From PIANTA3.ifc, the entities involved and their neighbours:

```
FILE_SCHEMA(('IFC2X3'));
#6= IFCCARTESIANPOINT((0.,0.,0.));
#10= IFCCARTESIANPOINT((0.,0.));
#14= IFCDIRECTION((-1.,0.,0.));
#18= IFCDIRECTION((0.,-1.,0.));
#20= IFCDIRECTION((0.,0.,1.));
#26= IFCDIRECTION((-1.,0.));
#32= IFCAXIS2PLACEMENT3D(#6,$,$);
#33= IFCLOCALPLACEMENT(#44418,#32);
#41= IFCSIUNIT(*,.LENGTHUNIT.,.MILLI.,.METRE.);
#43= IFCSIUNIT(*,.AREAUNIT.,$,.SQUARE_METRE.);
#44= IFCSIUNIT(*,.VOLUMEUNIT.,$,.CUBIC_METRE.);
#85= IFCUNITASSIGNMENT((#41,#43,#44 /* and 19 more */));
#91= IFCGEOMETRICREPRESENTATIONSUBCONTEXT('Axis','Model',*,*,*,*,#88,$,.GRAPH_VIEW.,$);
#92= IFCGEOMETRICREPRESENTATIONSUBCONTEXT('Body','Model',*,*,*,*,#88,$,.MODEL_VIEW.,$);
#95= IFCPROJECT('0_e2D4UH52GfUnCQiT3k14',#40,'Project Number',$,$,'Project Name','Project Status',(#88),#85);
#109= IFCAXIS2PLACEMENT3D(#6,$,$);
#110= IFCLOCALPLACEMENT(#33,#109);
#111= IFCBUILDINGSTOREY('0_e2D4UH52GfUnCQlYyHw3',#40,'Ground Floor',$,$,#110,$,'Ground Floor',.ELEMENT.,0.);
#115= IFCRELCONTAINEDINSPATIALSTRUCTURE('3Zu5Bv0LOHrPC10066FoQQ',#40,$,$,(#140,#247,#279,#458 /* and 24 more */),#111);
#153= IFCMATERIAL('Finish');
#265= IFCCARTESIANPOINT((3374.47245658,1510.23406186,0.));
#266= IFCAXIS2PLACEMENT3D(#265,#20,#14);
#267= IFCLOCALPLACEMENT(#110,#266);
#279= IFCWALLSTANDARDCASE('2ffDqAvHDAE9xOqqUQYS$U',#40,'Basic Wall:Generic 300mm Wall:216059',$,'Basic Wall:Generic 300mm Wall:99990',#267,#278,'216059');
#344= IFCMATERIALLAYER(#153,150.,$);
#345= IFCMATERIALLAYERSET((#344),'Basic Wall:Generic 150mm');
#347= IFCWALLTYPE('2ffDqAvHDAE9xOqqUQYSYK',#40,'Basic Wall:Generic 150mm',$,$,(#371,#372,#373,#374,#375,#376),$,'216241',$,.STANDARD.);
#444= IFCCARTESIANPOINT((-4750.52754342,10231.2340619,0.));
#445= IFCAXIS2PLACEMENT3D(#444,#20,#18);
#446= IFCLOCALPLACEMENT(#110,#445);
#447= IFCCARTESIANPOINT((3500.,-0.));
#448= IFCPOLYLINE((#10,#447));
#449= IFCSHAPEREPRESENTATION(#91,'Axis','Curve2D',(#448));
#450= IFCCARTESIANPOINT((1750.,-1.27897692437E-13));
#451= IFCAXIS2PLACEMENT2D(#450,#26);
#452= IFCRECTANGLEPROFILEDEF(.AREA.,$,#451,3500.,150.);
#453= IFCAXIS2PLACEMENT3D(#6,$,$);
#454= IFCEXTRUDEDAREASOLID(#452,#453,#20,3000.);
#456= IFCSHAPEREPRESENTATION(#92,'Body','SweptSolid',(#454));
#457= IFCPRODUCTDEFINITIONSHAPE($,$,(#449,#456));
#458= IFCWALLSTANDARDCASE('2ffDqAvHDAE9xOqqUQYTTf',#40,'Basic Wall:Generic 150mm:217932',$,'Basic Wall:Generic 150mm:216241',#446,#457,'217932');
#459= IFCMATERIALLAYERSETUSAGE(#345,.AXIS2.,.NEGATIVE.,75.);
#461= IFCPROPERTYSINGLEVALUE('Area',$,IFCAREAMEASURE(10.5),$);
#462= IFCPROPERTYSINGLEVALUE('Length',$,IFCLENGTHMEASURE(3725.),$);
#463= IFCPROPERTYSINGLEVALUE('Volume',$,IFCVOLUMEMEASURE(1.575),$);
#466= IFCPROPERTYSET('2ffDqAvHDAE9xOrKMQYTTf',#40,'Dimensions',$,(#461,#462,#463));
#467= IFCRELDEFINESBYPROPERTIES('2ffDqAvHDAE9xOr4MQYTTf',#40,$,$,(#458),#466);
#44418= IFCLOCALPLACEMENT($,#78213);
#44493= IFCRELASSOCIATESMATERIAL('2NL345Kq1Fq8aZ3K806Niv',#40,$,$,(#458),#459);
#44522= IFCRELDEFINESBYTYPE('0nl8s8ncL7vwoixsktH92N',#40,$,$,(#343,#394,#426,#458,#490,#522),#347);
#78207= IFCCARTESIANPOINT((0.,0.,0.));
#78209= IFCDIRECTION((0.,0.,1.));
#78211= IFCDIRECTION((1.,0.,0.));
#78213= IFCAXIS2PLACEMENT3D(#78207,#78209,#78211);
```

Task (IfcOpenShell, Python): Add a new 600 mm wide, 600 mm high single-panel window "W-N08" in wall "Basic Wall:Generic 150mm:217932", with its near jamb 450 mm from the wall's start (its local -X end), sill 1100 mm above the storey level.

```python
import numpy as np
import ifcopenshell
import ifcopenshell.api.feature
import ifcopenshell.api.geometry
import ifcopenshell.api.pset
import ifcopenshell.api.root
import ifcopenshell.api.spatial
import ifcopenshell.api.type
import ifcopenshell.geom
import ifcopenshell.util.element
import ifcopenshell.util.placement
import ifcopenshell.util.representation
import ifcopenshell.util.shape
import ifcopenshell.util.unit

model = ifcopenshell.open("PIANTA3.ifc")
unit_scale = ifcopenshell.util.unit.calculate_unit_scale(model)
area_scale = ifcopenshell.util.unit.calculate_unit_scale(model, "AREAUNIT")
volume_scale = ifcopenshell.util.unit.calculate_unit_scale(model, "VOLUMEUNIT")
settings = ifcopenshell.geom.settings()


def volume(element):
    """Net volume in cubic metres, openings subtracted."""
    shape = ifcopenshell.geom.create_shape(settings, element)
    return ifcopenshell.util.shape.get_volume(shape.geometry)


wall = model.by_id(458)
storey = ifcopenshell.util.element.get_container(wall, ifc_class="IfcBuildingStorey")
context = ifcopenshell.util.representation.get_context(model, "Model", "Body", "MODEL_VIEW")
before = volume(wall)

width, height, from_end, sill = 0.6, 0.6, 0.45, 1.1  # metres

# The wall runs along its own X axis, and the end named is its -X end.
wall_shape = ifcopenshell.geom.create_shape(settings, wall)
x, y, z = ifcopenshell.util.shape.get_vertices(wall_shape.geometry).T
start = x.min() + from_end
face, thickness = float(y.min()), float(y.max() - y.min())
wall_matrix = ifcopenshell.util.placement.get_local_placement(wall.ObjectPlacement)
level = ifcopenshell.util.placement.get_local_placement(storey.ObjectPlacement)[2, 3]


def in_wall(x, y):
    """Placement at x, y metres in the wall's axes, at sill height."""
    matrix = wall_matrix.copy()
    matrix[:, 3] = wall_matrix @ np.array([x / unit_scale, y / unit_scale, 0.0, 1.0])
    matrix[2, 3] = level + sill / unit_scale
    return matrix


# Opening: a box that overshoots both wall faces by 50 mm.
opening = ifcopenshell.api.root.create_entity(model, ifc_class="IfcOpeningElement")
box = ifcopenshell.api.geometry.add_wall_representation(
    model, context=context, length=width, height=height, thickness=thickness + 0.1
)
ifcopenshell.api.geometry.assign_representation(model, product=opening, representation=box)
ifcopenshell.api.geometry.edit_object_placement(model, product=opening, matrix=in_wall(start, face - 0.05), is_si=False)
ifcopenshell.api.feature.add_feature(model, feature=opening, element=wall)

window = ifcopenshell.api.root.create_entity(model, ifc_class="IfcWindow", name="W-N08")
window.OverallWidth, window.OverallHeight = width / unit_scale, height / unit_scale
body = ifcopenshell.api.geometry.add_window_representation(
    model,
    context=context,
    overall_width=window.OverallWidth,
    overall_height=window.OverallHeight,
    partition_type="SINGLE_PANEL",
)
ifcopenshell.api.geometry.assign_representation(model, product=window, representation=body)
ifcopenshell.api.spatial.assign_container(model, products=[window], relating_structure=storey)
fills = ifcopenshell.api.feature.add_filling(model, opening=opening, element=window)
fills.OwnerHistory = window.OwnerHistory  # required in IFC2X3

# IFC2X3 keeps the operation on the window style.
style = ifcopenshell.api.root.create_entity(model, ifc_class="IfcWindowStyle", name="W-N08")
style.OperationType, style.ConstructionType = "SINGLE_PANEL", "NOTDEFINED"
style.ParameterTakesPrecedence = style.Sizeable = False
ifcopenshell.api.type.assign_type(model, related_objects=[window], relating_type=style)

# Centre the window in the wall's thickness.
ifcopenshell.api.geometry.edit_object_placement(model, product=window, matrix=in_wall(start, face), is_si=False)
window_shape = ifcopenshell.geom.create_shape(settings, window)
depth = ifcopenshell.util.shape.get_vertices(window_shape.geometry)[:, 1]
offset = face + thickness / 2 - (depth.min() + depth.max()) / 2
ifcopenshell.api.geometry.edit_object_placement(model, product=window, matrix=in_wall(start, offset), is_si=False)

after = volume(wall)

# Update the wall's stored quantities.
pset = model.by_id(ifcopenshell.util.element.get_pset(wall, "Dimensions", should_inherit=False)["id"])
ifcopenshell.api.pset.edit_pset(model, pset=pset, properties={
    "Area": model.create_entity("IfcAreaMeasure", after / thickness / area_scale),
    "Volume": model.create_entity("IfcVolumeMeasure", after / volume_scale),
})

print(f"wall volume {before:.3f} -> {after:.3f} m3")

model.write("PIANTA3_updated.ifc")
```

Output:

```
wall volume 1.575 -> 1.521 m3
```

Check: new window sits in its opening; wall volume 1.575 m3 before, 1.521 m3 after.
